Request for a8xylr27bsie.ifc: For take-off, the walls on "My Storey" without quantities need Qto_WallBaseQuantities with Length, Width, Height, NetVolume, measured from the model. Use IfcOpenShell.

First a look at what the model holds.

```python
import ifcopenshell
import ifcopenshell.util.element
import ifcopenshell.util.unit

model = ifcopenshell.open("a8xylr27bsie.ifc")
print(model.schema)
for unit_type in ("LENGTHUNIT", "AREAUNIT", "VOLUMEUNIT"):
    print(unit_type, ifcopenshell.util.unit.calculate_unit_scale(model, unit_type))
storey = next(s for s in model.by_type("IfcBuildingStorey") if s.Name == "My Storey")
walls = [e for e in ifcopenshell.util.element.get_decomposition(storey) if e.is_a("IfcWall")]
for e in sorted(walls, key=lambda e: e.id()):
    print(e.id(), e.is_a(), e.Name, list(ifcopenshell.util.element.get_psets(e, qtos_only=True)), sep=" | ")
```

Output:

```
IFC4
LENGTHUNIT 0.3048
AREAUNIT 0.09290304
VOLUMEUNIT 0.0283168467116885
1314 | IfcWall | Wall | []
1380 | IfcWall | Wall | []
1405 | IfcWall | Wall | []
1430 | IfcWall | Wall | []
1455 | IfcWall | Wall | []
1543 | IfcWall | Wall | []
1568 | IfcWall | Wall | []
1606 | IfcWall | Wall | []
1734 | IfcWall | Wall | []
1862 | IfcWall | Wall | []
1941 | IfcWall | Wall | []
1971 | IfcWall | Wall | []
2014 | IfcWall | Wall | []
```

```python
import ifcopenshell
import ifcopenshell.api.pset
import ifcopenshell.geom
import ifcopenshell.util.element
import ifcopenshell.util.shape
import ifcopenshell.util.unit

model = ifcopenshell.open("a8xylr27bsie.ifc")
unit_scale = ifcopenshell.util.unit.calculate_unit_scale(model)
volume_scale = ifcopenshell.util.unit.calculate_unit_scale(model, "VOLUMEUNIT")
settings = ifcopenshell.geom.settings()

storey = next(s for s in model.by_type("IfcBuildingStorey") if s.Name == "My Storey")
walls = [e for e in ifcopenshell.util.element.get_decomposition(storey) if e.is_a("IfcWall")]

for e in sorted(walls, key=lambda e: e.id()):
    if ifcopenshell.util.element.get_psets(e, qtos_only=True, should_inherit=False):
        continue
    # Geometry comes back in metres, in the element's own axes.
    shape = ifcopenshell.geom.create_shape(settings, e)
    values = {
        "Length": ifcopenshell.util.shape.get_x(shape.geometry) / unit_scale,
        "Width": ifcopenshell.util.shape.get_y(shape.geometry) / unit_scale,
        "Height": ifcopenshell.util.shape.get_z(shape.geometry) / unit_scale,
        "NetVolume": ifcopenshell.util.shape.get_volume(shape.geometry) / volume_scale,
    }
    qto = ifcopenshell.api.pset.add_qto(model, product=e, name="Qto_WallBaseQuantities")
    ifcopenshell.api.pset.edit_qto(model, qto=qto, properties=values)
    print(e.id(), {k: round(v, 3) for k, v in values.items()})

model.write("a8xylr27bsie_rev.ifc")
```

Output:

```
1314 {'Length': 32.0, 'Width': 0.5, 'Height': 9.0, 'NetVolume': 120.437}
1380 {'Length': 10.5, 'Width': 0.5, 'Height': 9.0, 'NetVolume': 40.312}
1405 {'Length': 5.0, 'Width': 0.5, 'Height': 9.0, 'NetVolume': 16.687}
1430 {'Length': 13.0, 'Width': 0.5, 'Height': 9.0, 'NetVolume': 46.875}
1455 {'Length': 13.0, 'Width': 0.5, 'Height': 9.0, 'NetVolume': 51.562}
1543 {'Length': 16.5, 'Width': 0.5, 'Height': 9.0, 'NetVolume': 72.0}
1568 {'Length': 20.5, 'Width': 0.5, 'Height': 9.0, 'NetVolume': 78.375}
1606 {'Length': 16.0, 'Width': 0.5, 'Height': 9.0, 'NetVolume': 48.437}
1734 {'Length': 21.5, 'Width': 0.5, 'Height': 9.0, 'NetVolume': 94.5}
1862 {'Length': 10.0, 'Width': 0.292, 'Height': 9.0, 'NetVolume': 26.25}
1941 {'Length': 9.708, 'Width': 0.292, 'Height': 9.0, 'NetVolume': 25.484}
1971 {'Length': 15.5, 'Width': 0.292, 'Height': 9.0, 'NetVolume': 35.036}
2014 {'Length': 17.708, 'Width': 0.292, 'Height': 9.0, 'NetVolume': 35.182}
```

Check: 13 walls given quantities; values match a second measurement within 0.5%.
